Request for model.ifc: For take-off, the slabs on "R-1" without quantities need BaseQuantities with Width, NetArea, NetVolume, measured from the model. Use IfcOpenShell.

First a look at what the model holds.

```python
import ifcopenshell
import ifcopenshell.util.element
import ifcopenshell.util.unit

model = ifcopenshell.open("model.ifc")
print(model.schema)
for unit_type in ("LENGTHUNIT", "AREAUNIT", "VOLUMEUNIT"):
    print(unit_type, ifcopenshell.util.unit.calculate_unit_scale(model, unit_type))
storey = next(s for s in model.by_type("IfcBuildingStorey") if s.Name == "R-1")
slabs = [e for e in ifcopenshell.util.element.get_decomposition(storey) if e.is_a("IfcSlab")]
for e in sorted(slabs, key=lambda e: e.id()):
    print(e.id(), e.is_a(), e.Name, list(ifcopenshell.util.element.get_psets(e, qtos_only=True)), sep=" | ")
```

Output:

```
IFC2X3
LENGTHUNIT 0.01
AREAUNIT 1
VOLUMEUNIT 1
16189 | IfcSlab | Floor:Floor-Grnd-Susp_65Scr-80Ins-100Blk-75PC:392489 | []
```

```python
import ifcopenshell
import ifcopenshell.api.pset
import ifcopenshell.geom
import ifcopenshell.util.element
import ifcopenshell.util.shape
import ifcopenshell.util.unit

model = ifcopenshell.open("model.ifc")
unit_scale = ifcopenshell.util.unit.calculate_unit_scale(model)
area_scale = ifcopenshell.util.unit.calculate_unit_scale(model, "AREAUNIT")
volume_scale = ifcopenshell.util.unit.calculate_unit_scale(model, "VOLUMEUNIT")
settings = ifcopenshell.geom.settings()

storey = next(s for s in model.by_type("IfcBuildingStorey") if s.Name == "R-1")
slabs = [e for e in ifcopenshell.util.element.get_decomposition(storey) if e.is_a("IfcSlab")]

for e in sorted(slabs, key=lambda e: e.id()):
    if ifcopenshell.util.element.get_psets(e, qtos_only=True, should_inherit=False):
        continue
    # Geometry comes back in metres, in the element's own axes.
    shape = ifcopenshell.geom.create_shape(settings, e)
    values = {
        "Width": ifcopenshell.util.shape.get_z(shape.geometry) / unit_scale,
        "NetArea": ifcopenshell.util.shape.get_footprint_area(shape.geometry) / area_scale,
        "NetVolume": ifcopenshell.util.shape.get_volume(shape.geometry) / volume_scale,
    }
    qto = ifcopenshell.api.pset.add_qto(model, product=e, name="BaseQuantities")
    ifcopenshell.api.pset.edit_qto(model, qto=qto, properties=values)
    print(e.id(), {k: round(v, 3) for k, v in values.items()})

model.write("model_rev.ifc")
```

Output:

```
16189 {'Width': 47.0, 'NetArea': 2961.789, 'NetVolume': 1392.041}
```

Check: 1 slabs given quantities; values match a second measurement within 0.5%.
